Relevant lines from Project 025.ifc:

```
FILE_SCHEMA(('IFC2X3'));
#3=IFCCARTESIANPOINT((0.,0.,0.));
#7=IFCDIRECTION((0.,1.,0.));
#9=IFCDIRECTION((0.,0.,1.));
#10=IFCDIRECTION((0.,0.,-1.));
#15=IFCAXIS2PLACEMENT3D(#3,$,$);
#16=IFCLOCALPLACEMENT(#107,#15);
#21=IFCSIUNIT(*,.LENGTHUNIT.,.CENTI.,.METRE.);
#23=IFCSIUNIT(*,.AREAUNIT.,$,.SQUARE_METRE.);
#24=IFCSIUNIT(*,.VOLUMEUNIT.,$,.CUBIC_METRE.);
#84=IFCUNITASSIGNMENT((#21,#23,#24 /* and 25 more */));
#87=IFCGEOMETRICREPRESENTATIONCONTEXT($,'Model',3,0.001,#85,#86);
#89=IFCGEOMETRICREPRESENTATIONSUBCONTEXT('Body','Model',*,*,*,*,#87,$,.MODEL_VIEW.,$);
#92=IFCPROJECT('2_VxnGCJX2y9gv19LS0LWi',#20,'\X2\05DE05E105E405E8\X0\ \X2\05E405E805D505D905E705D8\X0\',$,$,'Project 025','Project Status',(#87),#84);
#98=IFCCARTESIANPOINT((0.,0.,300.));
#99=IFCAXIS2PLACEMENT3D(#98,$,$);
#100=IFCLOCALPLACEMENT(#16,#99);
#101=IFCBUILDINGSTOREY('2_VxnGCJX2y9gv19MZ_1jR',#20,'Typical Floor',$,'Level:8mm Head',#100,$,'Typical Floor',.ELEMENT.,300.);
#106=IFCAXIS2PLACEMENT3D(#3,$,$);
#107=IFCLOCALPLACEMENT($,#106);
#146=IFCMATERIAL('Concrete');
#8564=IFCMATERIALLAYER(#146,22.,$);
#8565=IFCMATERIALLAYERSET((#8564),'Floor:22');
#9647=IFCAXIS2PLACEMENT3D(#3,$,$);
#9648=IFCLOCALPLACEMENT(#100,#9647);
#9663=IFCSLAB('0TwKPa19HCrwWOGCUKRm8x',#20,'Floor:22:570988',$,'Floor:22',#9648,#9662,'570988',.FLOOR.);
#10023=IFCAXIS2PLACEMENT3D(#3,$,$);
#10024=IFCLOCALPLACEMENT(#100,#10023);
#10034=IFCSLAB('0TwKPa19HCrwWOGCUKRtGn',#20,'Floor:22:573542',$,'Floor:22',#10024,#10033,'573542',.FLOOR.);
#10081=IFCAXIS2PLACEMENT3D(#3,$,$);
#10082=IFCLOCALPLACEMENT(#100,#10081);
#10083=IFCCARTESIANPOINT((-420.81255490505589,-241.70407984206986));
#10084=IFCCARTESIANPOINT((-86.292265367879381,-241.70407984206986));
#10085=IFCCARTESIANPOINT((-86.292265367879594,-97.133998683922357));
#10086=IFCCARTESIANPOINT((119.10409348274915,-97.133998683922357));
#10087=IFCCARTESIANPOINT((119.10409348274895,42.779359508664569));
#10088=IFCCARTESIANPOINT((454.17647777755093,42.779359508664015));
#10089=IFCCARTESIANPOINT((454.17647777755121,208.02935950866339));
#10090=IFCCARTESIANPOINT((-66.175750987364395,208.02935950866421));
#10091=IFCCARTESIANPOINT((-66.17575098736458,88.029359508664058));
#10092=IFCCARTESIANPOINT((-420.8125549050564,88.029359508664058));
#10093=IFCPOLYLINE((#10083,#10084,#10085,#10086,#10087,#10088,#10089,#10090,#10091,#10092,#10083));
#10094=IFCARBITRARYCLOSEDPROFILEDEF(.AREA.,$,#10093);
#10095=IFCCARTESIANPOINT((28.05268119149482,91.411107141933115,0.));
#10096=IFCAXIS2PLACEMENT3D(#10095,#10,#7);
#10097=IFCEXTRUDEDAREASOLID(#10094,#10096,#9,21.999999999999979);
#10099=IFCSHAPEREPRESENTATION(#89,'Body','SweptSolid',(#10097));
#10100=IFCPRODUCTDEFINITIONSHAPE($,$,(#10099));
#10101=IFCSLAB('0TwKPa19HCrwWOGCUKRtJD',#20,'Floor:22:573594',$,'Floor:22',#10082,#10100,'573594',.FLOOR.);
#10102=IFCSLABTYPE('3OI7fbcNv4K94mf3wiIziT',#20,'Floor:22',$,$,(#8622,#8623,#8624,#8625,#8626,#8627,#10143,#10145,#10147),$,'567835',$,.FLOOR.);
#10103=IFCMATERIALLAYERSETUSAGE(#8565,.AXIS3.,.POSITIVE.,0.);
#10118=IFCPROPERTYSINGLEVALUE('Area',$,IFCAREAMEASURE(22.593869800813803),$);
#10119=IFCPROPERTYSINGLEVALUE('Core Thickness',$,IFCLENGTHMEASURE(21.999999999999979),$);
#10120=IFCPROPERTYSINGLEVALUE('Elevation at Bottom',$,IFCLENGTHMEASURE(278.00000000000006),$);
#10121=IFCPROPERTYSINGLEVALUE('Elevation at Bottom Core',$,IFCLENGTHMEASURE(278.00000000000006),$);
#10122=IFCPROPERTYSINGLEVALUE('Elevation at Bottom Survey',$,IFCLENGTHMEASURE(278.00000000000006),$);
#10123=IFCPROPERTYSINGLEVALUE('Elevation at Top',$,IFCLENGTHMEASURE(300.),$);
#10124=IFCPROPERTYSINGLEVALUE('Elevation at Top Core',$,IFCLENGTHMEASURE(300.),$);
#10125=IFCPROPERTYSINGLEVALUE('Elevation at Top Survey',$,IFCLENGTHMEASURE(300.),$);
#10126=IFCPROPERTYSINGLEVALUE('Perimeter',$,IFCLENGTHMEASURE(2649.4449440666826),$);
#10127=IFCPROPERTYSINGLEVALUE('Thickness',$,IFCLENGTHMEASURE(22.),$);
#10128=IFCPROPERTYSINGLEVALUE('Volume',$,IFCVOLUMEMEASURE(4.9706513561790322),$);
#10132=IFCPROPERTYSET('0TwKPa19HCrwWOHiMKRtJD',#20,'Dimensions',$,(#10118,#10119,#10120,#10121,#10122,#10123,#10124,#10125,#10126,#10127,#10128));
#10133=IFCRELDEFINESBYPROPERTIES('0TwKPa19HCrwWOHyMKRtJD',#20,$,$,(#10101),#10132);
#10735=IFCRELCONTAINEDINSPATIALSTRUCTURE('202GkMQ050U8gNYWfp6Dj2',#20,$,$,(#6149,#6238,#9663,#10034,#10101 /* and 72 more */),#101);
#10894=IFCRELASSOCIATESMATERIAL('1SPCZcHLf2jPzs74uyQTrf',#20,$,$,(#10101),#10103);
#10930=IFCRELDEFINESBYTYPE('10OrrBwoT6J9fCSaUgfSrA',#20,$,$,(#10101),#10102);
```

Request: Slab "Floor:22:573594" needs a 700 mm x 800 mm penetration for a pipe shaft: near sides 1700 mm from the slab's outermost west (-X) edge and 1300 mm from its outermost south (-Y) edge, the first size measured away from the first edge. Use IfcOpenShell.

```python
import numpy as np
import ifcopenshell
import ifcopenshell.api.feature
import ifcopenshell.api.geometry
import ifcopenshell.api.pset
import ifcopenshell.api.root
import ifcopenshell.geom
import ifcopenshell.util.element
import ifcopenshell.util.placement
import ifcopenshell.util.representation
import ifcopenshell.util.shape
import ifcopenshell.util.unit

model = ifcopenshell.open("Project 025.ifc")
unit_scale = ifcopenshell.util.unit.calculate_unit_scale(model)
area_scale = ifcopenshell.util.unit.calculate_unit_scale(model, "AREAUNIT")
volume_scale = ifcopenshell.util.unit.calculate_unit_scale(model, "VOLUMEUNIT")
settings = ifcopenshell.geom.settings()


def volume(element):
    """Net volume in cubic metres, openings subtracted."""
    shape = ifcopenshell.geom.create_shape(settings, element)
    return ifcopenshell.util.shape.get_volume(shape.geometry)


slab = model.by_id(10101)
before = volume(slab)

# Extent in the slab's own axes, in metres. The edges named are its -X and -Y sides.
slab_shape = ifcopenshell.geom.create_shape(settings, slab)
vertices = ifcopenshell.util.shape.get_vertices(slab_shape.geometry)
x_min, y_min, bottom = vertices.min(axis=0)
top = vertices[:, 2].max()

opening = ifcopenshell.api.root.create_entity(model, ifc_class="IfcOpeningElement", name="Pipe shaft opening")
context = ifcopenshell.util.representation.get_context(model, "Model", "Body", "MODEL_VIEW")
width, depth = 0.7, 0.8
outline = [(0.0, 0.0), (width, 0.0), (width, depth), (0.0, depth), (0.0, 0.0)]
# Overshoot both faces by 50 mm so the cut is clean.
shape = ifcopenshell.api.geometry.add_slab_representation(
    model, context=context, depth=top - bottom + 0.1, polyline=outline
)
ifcopenshell.api.geometry.assign_representation(model, product=opening, representation=shape)

matrix = ifcopenshell.util.placement.get_local_placement(slab.ObjectPlacement)
matrix[:, 3] = matrix @ np.append(np.array([x_min + 1.7, y_min + 1.3, bottom - 0.05]) / unit_scale, 1.0)
ifcopenshell.api.geometry.edit_object_placement(model, product=opening, matrix=matrix, is_si=False)
ifcopenshell.api.feature.add_feature(model, feature=opening, element=slab)

after = volume(slab)

# Update the slab's stored quantities.
pset = model.by_id(ifcopenshell.util.element.get_pset(slab, "Dimensions", should_inherit=False)["id"])
ifcopenshell.api.pset.edit_pset(model, pset=pset, properties={
    "Area": model.create_entity("IfcAreaMeasure", after / (top - bottom) / area_scale),
    "Volume": model.create_entity("IfcVolumeMeasure", after / volume_scale),
})

print(f"slab volume {before:.3f} -> {after:.3f} m3")

model.write("Project 025_updated.ifc")
```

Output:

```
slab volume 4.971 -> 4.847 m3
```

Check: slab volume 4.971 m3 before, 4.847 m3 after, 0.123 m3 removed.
